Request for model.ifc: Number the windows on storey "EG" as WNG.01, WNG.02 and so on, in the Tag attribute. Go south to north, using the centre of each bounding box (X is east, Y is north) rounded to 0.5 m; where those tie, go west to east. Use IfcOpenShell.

First a look at what the model holds.

```python
import ifcopenshell
import ifcopenshell.util.element
import ifcopenshell.util.placement

model = ifcopenshell.open("model.ifc")
print(model.schema)
storey = next(s for s in model.by_type("IfcBuildingStorey") if s.Name == "EG")
windows = [e for e in ifcopenshell.util.element.get_decomposition(storey) if e.is_a("IfcWindow")]
for e in sorted(windows, key=lambda e: e.id()):
    origin = ifcopenshell.util.placement.get_local_placement(e.ObjectPlacement)[:3, 3]
    print(e.id(), e.Tag, e.Name, origin.round(2) + 0.0, sep=" | ")
```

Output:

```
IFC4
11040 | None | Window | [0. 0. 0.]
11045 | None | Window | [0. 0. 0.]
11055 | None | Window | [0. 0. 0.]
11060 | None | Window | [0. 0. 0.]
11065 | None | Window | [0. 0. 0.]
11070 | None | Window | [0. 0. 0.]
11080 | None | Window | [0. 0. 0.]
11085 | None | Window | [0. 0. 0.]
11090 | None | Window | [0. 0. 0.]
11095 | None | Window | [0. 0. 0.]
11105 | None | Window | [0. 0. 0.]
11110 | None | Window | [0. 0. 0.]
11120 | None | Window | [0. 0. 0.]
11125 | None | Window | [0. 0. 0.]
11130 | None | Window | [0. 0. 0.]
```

```python
import ifcopenshell
import ifcopenshell.geom
import ifcopenshell.util.element
import ifcopenshell.util.shape

model = ifcopenshell.open("model.ifc")
settings = ifcopenshell.geom.settings()
settings.set("use-world-coords", True)


def centre(element):
    shape = ifcopenshell.geom.create_shape(settings, element)
    return ifcopenshell.util.shape.get_bbox_centroid(shape.geometry)


storey = next(s for s in model.by_type("IfcBuildingStorey") if s.Name == "EG")
windows = [e for e in ifcopenshell.util.element.get_decomposition(storey) if e.is_a("IfcWindow")]

# Insertion points can sit at a corner or the storey origin, so sort by the geometry (in metres).
centres = {e: centre(e) for e in windows}
windows.sort(key=lambda e: (round(centres[e][1] / 0.5), centres[e][0]))

for i, e in enumerate(windows, start=1):
    number = f"WNG.{i:02d}"
    e.Tag = number
    print(e.id(), number)

model.write("model-out.ifc")
```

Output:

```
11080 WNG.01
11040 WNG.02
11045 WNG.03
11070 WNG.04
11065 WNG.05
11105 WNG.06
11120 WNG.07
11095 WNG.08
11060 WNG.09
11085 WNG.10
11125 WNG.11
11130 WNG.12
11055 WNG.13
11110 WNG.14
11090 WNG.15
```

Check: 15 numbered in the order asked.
